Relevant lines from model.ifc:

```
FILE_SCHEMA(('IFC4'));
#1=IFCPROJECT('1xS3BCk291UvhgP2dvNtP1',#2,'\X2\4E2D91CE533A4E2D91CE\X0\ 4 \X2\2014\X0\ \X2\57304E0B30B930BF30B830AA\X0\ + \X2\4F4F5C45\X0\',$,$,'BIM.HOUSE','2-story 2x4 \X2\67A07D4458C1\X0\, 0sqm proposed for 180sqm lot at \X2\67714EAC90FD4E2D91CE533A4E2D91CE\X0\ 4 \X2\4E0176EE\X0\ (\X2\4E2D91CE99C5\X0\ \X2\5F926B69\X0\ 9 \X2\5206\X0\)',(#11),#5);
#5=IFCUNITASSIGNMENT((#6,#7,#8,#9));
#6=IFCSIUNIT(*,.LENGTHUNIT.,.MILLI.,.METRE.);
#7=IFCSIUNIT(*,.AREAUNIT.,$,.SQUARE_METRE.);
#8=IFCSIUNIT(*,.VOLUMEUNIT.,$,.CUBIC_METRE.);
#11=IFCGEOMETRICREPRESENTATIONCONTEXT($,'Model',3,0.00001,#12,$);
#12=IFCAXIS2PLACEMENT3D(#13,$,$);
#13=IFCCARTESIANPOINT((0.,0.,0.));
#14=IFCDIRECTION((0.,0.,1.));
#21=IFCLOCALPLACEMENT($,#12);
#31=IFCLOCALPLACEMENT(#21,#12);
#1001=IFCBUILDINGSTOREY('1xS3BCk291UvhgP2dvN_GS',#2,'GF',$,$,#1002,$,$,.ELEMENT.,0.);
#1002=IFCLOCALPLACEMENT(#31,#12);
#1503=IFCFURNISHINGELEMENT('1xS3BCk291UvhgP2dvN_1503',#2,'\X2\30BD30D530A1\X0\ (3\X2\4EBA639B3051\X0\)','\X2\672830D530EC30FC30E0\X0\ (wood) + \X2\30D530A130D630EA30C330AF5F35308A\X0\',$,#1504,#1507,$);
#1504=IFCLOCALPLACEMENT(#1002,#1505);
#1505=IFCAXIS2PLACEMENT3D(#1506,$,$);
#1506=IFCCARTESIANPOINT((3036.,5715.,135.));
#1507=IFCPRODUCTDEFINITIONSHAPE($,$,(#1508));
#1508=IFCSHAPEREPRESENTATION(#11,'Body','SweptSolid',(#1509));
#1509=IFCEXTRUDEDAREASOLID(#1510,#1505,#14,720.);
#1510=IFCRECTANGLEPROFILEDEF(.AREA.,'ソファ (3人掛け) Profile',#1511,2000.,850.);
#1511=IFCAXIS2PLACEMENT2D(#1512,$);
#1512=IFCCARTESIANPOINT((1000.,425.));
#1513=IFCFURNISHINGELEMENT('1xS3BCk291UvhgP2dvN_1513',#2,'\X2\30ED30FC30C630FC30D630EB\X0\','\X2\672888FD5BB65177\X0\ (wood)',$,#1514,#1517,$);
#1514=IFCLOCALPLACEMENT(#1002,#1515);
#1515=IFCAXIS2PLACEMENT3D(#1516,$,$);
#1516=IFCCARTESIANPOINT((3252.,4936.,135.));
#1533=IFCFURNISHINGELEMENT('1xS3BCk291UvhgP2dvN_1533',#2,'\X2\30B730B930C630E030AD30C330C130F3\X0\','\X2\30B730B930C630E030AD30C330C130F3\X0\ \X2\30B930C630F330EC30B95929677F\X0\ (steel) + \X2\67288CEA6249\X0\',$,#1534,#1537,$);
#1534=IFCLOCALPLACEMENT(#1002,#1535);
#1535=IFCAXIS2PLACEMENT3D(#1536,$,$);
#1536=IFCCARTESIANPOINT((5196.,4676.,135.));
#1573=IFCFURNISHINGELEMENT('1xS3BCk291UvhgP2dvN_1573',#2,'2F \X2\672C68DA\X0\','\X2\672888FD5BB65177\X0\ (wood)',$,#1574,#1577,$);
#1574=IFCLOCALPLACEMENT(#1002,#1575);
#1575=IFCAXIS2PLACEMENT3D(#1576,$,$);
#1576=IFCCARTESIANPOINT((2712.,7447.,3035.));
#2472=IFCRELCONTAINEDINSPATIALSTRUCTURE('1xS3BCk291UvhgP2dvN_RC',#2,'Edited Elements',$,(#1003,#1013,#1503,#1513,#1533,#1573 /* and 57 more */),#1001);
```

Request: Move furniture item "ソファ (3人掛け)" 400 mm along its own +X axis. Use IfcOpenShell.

```python
import ifcopenshell
import ifcopenshell.api.geometry
import ifcopenshell.util.placement
import ifcopenshell.util.unit

model = ifcopenshell.open("model.ifc")
unit_scale = ifcopenshell.util.unit.calculate_unit_scale(model)

item = model.by_id(1503)
matrix = ifcopenshell.util.placement.get_local_placement(item.ObjectPlacement)
matrix[:3, 3] += matrix[:3, 0] * 0.4 / unit_scale
ifcopenshell.api.geometry.edit_object_placement(model, product=item, matrix=matrix, is_si=False)

print(ifcopenshell.util.placement.get_local_placement(item.ObjectPlacement).round(3) + 0.0)

model.write("model_v2.ifc")
```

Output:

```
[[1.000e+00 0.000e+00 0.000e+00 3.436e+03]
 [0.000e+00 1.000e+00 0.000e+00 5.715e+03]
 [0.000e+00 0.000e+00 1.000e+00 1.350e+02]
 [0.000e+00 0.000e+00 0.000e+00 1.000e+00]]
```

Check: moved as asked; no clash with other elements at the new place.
